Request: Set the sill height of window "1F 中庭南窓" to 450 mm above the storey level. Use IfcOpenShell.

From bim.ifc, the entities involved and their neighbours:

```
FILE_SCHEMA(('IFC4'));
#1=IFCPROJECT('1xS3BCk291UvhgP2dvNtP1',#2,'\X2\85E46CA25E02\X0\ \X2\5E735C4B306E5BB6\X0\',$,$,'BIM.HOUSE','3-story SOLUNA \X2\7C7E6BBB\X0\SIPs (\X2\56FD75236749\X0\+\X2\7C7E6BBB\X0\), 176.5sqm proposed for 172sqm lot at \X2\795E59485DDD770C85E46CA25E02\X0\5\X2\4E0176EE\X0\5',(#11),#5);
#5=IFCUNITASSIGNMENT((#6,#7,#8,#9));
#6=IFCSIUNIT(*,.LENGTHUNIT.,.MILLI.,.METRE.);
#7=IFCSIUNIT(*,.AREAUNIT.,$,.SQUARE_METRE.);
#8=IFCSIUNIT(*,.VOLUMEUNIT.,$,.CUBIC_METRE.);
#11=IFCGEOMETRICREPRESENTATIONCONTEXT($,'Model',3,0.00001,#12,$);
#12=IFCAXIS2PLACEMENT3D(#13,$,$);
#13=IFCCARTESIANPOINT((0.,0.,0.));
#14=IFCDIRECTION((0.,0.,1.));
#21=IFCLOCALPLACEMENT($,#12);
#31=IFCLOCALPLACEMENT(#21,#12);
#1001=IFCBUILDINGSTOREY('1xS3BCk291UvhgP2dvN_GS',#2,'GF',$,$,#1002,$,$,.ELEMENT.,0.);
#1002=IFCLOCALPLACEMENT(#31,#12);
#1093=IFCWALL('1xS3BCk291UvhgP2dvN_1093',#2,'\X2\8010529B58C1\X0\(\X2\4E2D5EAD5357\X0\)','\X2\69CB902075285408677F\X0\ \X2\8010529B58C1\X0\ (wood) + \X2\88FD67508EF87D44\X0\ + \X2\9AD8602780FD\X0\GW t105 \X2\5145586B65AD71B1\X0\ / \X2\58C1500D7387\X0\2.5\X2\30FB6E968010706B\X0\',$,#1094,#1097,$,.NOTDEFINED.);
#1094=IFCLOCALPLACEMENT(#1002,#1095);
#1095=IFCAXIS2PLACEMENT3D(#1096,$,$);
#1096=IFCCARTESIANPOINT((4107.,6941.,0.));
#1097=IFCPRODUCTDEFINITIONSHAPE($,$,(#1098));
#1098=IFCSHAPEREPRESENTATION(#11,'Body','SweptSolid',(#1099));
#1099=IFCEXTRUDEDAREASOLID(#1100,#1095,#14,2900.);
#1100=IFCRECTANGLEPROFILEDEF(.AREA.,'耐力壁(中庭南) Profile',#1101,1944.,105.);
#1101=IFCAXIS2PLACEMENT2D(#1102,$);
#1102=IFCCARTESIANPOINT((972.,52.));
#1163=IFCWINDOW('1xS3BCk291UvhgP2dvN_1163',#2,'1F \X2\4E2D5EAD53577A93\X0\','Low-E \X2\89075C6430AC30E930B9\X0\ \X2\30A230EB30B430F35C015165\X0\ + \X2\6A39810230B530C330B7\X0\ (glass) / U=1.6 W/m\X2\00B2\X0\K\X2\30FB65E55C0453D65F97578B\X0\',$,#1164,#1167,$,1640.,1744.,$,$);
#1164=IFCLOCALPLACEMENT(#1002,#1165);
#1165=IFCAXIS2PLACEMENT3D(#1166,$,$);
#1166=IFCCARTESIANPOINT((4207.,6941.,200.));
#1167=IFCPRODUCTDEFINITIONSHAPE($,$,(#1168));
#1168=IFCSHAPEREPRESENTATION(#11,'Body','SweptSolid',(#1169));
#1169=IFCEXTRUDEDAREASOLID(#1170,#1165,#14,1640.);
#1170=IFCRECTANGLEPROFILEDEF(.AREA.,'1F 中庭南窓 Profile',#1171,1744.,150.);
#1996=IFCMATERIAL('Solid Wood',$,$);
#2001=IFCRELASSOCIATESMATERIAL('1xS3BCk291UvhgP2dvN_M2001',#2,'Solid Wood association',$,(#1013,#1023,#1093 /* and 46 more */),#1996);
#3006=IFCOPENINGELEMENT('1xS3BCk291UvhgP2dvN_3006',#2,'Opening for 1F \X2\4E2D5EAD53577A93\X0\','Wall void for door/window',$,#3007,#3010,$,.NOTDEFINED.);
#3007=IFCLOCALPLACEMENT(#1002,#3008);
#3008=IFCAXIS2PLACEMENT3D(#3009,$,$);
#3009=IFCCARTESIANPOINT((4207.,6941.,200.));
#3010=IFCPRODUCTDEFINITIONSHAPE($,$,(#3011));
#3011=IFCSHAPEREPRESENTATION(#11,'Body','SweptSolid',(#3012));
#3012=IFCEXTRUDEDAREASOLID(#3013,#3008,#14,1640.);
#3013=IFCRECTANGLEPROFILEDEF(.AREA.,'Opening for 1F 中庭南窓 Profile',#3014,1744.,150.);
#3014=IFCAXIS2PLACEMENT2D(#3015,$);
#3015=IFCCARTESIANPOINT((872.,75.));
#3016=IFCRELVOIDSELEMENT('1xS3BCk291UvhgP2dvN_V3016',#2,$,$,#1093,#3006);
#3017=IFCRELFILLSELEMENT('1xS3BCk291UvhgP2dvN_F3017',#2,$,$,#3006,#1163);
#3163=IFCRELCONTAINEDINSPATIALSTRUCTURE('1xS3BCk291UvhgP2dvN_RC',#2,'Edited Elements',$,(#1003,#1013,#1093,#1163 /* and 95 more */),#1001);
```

```python
import numpy as np
import ifcopenshell
import ifcopenshell.api.geometry
import ifcopenshell.geom
import ifcopenshell.util.element
import ifcopenshell.util.placement
import ifcopenshell.util.shape
import ifcopenshell.util.unit

model = ifcopenshell.open("bim.ifc")
unit_scale = ifcopenshell.util.unit.calculate_unit_scale(model)

window = model.by_guid("1xS3BCk291UvhgP2dvN_1163")
opening = window.FillsVoids[0].RelatingOpeningElement
storey = ifcopenshell.util.element.get_container(window, ifc_class="IfcBuildingStorey")
level = ifcopenshell.util.placement.get_local_placement(storey.ObjectPlacement)[2, 3]

# The opening's origin need not be at the sill, so measure its lowest point.
shape = ifcopenshell.geom.create_shape(ifcopenshell.geom.settings(), opening)
bottom = ifcopenshell.util.shape.get_shape_bottom_elevation(shape, shape.geometry) / unit_scale
dz = level + 0.45 / unit_scale - bottom

shift = np.array([0.0, 0.0, dz])
# The window is not placed relative to its opening, so move both.
for product in (opening, window):
    matrix = ifcopenshell.util.placement.get_local_placement(product.ObjectPlacement)
    matrix[:3, 3] += shift
    ifcopenshell.api.geometry.edit_object_placement(model, product=product, matrix=matrix, is_si=False)

print(f"moved by {dz * unit_scale:+.3f} m")

model.write("bim_rev.ifc")
```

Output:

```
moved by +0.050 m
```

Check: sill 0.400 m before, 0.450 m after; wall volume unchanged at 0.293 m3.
